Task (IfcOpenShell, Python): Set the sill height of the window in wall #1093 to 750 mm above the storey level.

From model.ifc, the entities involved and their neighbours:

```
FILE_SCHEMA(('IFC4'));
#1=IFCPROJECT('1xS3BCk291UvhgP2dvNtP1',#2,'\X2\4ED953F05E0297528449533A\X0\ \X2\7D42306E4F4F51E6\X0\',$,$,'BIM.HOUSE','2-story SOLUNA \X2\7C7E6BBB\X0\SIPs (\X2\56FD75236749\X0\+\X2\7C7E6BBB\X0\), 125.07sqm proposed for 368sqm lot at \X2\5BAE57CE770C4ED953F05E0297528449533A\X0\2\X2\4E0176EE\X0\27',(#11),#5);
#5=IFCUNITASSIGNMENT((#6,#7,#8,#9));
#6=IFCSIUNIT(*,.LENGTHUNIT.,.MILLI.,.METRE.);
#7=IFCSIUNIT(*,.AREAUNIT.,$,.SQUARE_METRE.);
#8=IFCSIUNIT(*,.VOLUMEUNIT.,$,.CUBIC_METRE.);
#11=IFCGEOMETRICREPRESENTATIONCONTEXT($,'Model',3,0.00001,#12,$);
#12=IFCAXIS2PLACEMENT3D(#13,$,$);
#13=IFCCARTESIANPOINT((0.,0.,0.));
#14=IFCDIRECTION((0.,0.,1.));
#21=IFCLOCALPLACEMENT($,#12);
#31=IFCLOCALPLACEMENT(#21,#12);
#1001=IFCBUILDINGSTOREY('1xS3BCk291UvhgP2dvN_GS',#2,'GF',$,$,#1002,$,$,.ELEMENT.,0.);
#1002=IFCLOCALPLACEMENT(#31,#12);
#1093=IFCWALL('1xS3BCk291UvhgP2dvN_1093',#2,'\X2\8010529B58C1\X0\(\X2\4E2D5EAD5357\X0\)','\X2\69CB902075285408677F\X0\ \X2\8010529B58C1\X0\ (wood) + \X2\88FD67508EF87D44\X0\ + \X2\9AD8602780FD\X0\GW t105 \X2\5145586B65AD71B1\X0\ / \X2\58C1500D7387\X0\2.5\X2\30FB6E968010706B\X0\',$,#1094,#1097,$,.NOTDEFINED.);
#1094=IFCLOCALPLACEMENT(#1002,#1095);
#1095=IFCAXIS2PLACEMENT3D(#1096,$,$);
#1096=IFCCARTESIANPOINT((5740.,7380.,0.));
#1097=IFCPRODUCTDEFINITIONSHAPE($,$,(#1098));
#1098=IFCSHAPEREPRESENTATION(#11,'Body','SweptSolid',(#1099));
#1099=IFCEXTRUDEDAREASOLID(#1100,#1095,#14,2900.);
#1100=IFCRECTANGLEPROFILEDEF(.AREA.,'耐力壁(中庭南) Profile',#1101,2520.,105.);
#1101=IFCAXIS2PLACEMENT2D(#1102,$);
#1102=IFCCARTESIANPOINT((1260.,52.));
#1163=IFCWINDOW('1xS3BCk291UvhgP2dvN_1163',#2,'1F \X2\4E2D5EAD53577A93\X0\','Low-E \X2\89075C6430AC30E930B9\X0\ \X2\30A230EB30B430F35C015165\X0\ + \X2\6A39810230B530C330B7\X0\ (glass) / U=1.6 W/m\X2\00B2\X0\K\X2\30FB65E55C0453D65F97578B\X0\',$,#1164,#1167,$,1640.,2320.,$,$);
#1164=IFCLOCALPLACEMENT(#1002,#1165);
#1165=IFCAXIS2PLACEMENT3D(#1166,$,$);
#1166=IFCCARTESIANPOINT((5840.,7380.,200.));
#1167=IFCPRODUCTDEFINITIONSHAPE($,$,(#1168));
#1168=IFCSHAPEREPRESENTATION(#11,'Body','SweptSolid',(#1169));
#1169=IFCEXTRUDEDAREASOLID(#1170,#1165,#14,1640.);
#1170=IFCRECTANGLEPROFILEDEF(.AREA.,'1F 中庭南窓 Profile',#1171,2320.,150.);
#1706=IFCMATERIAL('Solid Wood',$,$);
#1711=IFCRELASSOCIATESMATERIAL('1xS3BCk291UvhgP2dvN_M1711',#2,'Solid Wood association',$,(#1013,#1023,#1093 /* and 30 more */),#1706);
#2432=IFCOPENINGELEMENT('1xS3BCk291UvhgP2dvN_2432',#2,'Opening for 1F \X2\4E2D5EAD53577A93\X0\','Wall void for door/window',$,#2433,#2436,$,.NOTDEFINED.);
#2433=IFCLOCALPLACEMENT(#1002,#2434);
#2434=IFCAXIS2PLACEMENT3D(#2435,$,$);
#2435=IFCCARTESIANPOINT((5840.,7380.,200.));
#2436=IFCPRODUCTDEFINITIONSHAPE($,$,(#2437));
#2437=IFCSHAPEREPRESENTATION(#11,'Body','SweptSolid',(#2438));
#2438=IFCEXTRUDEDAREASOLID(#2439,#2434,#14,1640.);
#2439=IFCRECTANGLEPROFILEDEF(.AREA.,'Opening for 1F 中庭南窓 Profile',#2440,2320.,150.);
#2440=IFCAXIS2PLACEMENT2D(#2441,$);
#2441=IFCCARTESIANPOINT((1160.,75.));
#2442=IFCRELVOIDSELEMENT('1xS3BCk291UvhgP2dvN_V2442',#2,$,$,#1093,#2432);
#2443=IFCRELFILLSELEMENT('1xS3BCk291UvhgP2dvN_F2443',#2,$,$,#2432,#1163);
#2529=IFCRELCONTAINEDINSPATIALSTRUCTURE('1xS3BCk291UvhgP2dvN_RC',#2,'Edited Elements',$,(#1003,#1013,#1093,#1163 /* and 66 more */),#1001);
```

```python
import numpy as np
import ifcopenshell
import ifcopenshell.api.geometry
import ifcopenshell.geom
import ifcopenshell.util.element
import ifcopenshell.util.placement
import ifcopenshell.util.shape
import ifcopenshell.util.unit

model = ifcopenshell.open("model.ifc")
unit_scale = ifcopenshell.util.unit.calculate_unit_scale(model)

window = model.by_id(1163)
opening = window.FillsVoids[0].RelatingOpeningElement
storey = ifcopenshell.util.element.get_container(window, ifc_class="IfcBuildingStorey")
level = ifcopenshell.util.placement.get_local_placement(storey.ObjectPlacement)[2, 3]

# The opening's origin need not be at the sill, so measure its lowest point.
shape = ifcopenshell.geom.create_shape(ifcopenshell.geom.settings(), opening)
bottom = ifcopenshell.util.shape.get_shape_bottom_elevation(shape, shape.geometry) / unit_scale
dz = level + 750.0 - bottom

shift = np.array([0.0, 0.0, dz])
# The window is not placed relative to its opening, so move both.
for product in (opening, window):
    matrix = ifcopenshell.util.placement.get_local_placement(product.ObjectPlacement)
    matrix[:3, 3] += shift
    ifcopenshell.api.geometry.edit_object_placement(model, product=product, matrix=matrix, is_si=False)

print(f"moved by {dz * unit_scale:+.3f} m")

model.write("model_v2.ifc")
```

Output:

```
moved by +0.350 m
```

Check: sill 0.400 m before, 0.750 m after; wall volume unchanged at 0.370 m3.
